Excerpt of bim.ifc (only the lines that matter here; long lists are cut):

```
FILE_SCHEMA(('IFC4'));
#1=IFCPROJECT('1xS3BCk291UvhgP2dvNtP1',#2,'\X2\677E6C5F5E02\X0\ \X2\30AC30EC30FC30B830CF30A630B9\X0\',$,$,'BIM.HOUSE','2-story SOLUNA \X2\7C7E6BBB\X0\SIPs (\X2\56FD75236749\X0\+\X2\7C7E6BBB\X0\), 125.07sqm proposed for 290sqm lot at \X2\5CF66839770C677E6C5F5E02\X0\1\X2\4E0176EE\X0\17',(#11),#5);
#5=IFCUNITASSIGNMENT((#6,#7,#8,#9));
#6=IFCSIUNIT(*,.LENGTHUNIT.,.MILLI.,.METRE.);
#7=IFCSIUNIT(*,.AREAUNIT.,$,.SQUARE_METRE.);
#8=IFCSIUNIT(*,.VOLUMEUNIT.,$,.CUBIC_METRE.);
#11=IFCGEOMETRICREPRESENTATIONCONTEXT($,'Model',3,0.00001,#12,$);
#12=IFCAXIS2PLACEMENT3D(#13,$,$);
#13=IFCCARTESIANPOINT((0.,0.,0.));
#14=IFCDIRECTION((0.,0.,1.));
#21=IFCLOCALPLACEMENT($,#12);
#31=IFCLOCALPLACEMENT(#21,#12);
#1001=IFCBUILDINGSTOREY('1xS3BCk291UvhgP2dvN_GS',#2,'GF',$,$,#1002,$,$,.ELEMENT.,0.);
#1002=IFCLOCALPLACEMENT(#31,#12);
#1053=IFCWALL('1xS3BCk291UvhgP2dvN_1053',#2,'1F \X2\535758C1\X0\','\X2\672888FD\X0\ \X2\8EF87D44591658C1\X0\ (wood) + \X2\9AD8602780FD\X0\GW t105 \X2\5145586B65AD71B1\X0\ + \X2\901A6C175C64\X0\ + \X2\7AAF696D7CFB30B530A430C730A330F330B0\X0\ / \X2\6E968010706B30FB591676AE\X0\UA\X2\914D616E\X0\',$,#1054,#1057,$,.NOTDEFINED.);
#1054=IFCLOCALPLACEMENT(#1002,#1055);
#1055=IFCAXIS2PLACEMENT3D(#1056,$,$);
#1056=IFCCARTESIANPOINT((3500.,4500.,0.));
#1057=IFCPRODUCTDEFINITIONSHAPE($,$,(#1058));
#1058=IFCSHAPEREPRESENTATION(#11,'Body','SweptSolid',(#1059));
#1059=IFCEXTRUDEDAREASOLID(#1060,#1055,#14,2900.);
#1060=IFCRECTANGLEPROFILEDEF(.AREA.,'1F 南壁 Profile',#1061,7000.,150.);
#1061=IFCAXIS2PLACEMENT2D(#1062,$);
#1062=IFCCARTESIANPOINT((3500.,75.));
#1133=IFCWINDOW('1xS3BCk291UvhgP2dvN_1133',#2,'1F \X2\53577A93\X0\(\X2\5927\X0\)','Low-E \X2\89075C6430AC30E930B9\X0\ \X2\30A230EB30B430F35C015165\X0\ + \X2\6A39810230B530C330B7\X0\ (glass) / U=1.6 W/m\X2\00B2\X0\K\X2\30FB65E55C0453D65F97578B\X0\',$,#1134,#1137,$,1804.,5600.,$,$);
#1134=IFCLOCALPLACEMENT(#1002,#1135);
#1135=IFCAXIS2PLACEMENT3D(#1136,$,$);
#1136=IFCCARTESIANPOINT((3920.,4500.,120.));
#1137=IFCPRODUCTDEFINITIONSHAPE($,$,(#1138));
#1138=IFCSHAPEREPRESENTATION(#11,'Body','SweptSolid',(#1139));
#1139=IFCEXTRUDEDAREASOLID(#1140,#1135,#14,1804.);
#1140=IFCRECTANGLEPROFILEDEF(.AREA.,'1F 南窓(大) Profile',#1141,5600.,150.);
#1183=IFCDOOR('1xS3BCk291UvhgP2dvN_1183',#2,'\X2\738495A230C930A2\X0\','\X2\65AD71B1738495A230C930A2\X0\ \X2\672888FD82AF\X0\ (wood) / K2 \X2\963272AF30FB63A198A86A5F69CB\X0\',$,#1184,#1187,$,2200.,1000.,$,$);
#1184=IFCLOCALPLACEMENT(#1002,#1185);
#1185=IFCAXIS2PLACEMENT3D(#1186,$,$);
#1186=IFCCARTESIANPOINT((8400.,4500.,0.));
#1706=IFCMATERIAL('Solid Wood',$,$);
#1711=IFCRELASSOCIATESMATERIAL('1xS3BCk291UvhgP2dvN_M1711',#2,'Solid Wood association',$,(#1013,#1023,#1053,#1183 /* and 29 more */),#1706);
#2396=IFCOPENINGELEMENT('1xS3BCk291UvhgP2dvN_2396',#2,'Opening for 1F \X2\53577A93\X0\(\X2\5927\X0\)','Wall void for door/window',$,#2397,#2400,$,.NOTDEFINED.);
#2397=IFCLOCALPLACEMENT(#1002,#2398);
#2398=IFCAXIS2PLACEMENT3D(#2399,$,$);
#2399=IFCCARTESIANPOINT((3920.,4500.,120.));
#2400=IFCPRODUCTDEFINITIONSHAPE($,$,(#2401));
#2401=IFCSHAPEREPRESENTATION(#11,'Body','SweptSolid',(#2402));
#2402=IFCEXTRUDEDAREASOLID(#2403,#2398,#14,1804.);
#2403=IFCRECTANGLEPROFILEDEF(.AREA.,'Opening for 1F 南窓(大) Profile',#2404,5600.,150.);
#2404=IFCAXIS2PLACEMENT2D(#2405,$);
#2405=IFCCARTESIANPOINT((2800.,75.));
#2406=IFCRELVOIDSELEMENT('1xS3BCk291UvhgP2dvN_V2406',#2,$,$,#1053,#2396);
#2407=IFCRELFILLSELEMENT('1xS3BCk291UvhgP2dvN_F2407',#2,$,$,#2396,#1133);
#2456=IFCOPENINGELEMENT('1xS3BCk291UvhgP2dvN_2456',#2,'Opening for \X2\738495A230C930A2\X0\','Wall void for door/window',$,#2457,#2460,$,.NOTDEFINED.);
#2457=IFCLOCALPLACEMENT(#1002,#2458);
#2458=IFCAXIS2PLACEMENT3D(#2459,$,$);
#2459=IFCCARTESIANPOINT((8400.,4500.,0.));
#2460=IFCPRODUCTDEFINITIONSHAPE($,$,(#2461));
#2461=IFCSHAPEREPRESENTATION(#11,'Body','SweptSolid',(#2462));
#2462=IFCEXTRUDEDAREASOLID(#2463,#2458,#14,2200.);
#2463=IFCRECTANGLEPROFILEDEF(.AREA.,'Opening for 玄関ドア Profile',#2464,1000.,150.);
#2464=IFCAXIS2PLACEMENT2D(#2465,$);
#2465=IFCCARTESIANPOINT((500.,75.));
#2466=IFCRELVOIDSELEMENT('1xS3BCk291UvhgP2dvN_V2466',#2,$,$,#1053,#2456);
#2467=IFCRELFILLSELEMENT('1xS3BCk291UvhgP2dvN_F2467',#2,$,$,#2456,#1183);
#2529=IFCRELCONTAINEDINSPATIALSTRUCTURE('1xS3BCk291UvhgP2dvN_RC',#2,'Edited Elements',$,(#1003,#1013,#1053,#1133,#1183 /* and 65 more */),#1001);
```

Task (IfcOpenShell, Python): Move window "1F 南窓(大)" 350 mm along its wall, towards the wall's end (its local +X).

```python
import ifcopenshell
import ifcopenshell.api.geometry
import ifcopenshell.util.placement
import ifcopenshell.util.unit

model = ifcopenshell.open("bim.ifc")
unit_scale = ifcopenshell.util.unit.calculate_unit_scale(model)

window = model.by_guid("1xS3BCk291UvhgP2dvN_1133")
opening = window.FillsVoids[0].RelatingOpeningElement
wall = opening.VoidsElements[0].RelatingBuildingElement

wall_matrix = ifcopenshell.util.placement.get_local_placement(wall.ObjectPlacement)
shift = wall_matrix[:3, 0] * 0.35 / unit_scale
before = ifcopenshell.util.placement.get_local_placement(window.ObjectPlacement)[:3, 3].copy()

# The window is not placed relative to its opening, so move both.
for product in (opening, window):
    matrix = ifcopenshell.util.placement.get_local_placement(product.ObjectPlacement)
    matrix[:3, 3] += shift
    ifcopenshell.api.geometry.edit_object_placement(model, product=product, matrix=matrix, is_si=False)

after = ifcopenshell.util.placement.get_local_placement(window.ObjectPlacement)[:3, 3]
print("window moved by", (after - before).round(3) + 0.0)

model.write("bim_rev.ifc")
```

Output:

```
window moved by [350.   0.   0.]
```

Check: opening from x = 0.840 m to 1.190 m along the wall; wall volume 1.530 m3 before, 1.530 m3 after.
